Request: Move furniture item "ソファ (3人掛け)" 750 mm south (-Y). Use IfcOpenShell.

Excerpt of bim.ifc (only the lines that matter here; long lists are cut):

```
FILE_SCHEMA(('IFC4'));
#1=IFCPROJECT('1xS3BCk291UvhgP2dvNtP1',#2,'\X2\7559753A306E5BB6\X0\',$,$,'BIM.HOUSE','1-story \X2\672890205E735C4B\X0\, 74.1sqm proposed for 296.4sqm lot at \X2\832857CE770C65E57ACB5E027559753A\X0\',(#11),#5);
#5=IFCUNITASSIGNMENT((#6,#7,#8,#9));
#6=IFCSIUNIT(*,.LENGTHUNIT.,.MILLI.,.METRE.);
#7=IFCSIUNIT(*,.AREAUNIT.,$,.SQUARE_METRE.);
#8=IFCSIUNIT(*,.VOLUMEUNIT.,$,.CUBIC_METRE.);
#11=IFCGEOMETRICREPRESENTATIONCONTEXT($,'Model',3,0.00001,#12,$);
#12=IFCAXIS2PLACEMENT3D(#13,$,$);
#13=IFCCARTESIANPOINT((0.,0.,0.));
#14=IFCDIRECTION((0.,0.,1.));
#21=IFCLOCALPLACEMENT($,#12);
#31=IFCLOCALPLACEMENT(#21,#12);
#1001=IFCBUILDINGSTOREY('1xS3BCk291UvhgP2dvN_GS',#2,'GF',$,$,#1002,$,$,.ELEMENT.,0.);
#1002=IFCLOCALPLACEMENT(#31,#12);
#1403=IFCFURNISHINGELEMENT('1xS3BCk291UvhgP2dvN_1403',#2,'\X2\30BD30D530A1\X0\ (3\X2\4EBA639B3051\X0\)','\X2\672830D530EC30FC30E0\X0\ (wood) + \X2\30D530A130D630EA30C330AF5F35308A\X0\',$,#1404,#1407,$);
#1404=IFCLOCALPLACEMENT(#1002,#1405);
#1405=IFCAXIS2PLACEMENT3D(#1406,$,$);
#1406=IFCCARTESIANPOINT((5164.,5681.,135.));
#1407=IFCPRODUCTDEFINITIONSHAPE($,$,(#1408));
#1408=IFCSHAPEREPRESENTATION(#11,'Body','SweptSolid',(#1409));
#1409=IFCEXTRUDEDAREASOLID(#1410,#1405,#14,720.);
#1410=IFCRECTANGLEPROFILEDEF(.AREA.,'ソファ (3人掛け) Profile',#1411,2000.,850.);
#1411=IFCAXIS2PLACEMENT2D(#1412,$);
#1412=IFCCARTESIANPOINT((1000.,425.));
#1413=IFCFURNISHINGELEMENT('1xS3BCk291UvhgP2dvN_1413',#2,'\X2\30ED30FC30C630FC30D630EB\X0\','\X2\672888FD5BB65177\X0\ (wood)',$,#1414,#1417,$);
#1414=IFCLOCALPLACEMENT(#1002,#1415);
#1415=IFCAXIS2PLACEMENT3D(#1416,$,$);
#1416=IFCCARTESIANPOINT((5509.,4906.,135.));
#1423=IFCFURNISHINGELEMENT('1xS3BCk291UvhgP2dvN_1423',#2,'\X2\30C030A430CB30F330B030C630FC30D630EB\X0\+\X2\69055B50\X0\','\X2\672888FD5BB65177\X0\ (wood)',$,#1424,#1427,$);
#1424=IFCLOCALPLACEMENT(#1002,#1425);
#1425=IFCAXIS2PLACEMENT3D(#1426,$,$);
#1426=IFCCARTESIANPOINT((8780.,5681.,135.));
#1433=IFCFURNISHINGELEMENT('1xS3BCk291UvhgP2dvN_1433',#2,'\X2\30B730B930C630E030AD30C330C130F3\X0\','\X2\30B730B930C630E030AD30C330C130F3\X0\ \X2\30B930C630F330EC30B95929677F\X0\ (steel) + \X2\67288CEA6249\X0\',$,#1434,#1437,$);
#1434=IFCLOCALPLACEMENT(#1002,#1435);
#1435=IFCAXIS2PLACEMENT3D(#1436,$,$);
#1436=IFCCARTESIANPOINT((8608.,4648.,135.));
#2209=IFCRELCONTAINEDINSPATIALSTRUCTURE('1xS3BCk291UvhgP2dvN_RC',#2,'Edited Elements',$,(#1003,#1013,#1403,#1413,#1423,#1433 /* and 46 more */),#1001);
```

```python
import ifcopenshell
import ifcopenshell.api.geometry
import ifcopenshell.util.placement

model = ifcopenshell.open("bim.ifc")

item = model.by_guid("1xS3BCk291UvhgP2dvN_1403")
matrix = ifcopenshell.util.placement.get_local_placement(item.ObjectPlacement)
matrix[1, 3] -= 750.0
ifcopenshell.api.geometry.edit_object_placement(model, product=item, matrix=matrix, is_si=False)

print(ifcopenshell.util.placement.get_local_placement(item.ObjectPlacement).round(3) + 0.0)

model.write("bim_updated.ifc")
```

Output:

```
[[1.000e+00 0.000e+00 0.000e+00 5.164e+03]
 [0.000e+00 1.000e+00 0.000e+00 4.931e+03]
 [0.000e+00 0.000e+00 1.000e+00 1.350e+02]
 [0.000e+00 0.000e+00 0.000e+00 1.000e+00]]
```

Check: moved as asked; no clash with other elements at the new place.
